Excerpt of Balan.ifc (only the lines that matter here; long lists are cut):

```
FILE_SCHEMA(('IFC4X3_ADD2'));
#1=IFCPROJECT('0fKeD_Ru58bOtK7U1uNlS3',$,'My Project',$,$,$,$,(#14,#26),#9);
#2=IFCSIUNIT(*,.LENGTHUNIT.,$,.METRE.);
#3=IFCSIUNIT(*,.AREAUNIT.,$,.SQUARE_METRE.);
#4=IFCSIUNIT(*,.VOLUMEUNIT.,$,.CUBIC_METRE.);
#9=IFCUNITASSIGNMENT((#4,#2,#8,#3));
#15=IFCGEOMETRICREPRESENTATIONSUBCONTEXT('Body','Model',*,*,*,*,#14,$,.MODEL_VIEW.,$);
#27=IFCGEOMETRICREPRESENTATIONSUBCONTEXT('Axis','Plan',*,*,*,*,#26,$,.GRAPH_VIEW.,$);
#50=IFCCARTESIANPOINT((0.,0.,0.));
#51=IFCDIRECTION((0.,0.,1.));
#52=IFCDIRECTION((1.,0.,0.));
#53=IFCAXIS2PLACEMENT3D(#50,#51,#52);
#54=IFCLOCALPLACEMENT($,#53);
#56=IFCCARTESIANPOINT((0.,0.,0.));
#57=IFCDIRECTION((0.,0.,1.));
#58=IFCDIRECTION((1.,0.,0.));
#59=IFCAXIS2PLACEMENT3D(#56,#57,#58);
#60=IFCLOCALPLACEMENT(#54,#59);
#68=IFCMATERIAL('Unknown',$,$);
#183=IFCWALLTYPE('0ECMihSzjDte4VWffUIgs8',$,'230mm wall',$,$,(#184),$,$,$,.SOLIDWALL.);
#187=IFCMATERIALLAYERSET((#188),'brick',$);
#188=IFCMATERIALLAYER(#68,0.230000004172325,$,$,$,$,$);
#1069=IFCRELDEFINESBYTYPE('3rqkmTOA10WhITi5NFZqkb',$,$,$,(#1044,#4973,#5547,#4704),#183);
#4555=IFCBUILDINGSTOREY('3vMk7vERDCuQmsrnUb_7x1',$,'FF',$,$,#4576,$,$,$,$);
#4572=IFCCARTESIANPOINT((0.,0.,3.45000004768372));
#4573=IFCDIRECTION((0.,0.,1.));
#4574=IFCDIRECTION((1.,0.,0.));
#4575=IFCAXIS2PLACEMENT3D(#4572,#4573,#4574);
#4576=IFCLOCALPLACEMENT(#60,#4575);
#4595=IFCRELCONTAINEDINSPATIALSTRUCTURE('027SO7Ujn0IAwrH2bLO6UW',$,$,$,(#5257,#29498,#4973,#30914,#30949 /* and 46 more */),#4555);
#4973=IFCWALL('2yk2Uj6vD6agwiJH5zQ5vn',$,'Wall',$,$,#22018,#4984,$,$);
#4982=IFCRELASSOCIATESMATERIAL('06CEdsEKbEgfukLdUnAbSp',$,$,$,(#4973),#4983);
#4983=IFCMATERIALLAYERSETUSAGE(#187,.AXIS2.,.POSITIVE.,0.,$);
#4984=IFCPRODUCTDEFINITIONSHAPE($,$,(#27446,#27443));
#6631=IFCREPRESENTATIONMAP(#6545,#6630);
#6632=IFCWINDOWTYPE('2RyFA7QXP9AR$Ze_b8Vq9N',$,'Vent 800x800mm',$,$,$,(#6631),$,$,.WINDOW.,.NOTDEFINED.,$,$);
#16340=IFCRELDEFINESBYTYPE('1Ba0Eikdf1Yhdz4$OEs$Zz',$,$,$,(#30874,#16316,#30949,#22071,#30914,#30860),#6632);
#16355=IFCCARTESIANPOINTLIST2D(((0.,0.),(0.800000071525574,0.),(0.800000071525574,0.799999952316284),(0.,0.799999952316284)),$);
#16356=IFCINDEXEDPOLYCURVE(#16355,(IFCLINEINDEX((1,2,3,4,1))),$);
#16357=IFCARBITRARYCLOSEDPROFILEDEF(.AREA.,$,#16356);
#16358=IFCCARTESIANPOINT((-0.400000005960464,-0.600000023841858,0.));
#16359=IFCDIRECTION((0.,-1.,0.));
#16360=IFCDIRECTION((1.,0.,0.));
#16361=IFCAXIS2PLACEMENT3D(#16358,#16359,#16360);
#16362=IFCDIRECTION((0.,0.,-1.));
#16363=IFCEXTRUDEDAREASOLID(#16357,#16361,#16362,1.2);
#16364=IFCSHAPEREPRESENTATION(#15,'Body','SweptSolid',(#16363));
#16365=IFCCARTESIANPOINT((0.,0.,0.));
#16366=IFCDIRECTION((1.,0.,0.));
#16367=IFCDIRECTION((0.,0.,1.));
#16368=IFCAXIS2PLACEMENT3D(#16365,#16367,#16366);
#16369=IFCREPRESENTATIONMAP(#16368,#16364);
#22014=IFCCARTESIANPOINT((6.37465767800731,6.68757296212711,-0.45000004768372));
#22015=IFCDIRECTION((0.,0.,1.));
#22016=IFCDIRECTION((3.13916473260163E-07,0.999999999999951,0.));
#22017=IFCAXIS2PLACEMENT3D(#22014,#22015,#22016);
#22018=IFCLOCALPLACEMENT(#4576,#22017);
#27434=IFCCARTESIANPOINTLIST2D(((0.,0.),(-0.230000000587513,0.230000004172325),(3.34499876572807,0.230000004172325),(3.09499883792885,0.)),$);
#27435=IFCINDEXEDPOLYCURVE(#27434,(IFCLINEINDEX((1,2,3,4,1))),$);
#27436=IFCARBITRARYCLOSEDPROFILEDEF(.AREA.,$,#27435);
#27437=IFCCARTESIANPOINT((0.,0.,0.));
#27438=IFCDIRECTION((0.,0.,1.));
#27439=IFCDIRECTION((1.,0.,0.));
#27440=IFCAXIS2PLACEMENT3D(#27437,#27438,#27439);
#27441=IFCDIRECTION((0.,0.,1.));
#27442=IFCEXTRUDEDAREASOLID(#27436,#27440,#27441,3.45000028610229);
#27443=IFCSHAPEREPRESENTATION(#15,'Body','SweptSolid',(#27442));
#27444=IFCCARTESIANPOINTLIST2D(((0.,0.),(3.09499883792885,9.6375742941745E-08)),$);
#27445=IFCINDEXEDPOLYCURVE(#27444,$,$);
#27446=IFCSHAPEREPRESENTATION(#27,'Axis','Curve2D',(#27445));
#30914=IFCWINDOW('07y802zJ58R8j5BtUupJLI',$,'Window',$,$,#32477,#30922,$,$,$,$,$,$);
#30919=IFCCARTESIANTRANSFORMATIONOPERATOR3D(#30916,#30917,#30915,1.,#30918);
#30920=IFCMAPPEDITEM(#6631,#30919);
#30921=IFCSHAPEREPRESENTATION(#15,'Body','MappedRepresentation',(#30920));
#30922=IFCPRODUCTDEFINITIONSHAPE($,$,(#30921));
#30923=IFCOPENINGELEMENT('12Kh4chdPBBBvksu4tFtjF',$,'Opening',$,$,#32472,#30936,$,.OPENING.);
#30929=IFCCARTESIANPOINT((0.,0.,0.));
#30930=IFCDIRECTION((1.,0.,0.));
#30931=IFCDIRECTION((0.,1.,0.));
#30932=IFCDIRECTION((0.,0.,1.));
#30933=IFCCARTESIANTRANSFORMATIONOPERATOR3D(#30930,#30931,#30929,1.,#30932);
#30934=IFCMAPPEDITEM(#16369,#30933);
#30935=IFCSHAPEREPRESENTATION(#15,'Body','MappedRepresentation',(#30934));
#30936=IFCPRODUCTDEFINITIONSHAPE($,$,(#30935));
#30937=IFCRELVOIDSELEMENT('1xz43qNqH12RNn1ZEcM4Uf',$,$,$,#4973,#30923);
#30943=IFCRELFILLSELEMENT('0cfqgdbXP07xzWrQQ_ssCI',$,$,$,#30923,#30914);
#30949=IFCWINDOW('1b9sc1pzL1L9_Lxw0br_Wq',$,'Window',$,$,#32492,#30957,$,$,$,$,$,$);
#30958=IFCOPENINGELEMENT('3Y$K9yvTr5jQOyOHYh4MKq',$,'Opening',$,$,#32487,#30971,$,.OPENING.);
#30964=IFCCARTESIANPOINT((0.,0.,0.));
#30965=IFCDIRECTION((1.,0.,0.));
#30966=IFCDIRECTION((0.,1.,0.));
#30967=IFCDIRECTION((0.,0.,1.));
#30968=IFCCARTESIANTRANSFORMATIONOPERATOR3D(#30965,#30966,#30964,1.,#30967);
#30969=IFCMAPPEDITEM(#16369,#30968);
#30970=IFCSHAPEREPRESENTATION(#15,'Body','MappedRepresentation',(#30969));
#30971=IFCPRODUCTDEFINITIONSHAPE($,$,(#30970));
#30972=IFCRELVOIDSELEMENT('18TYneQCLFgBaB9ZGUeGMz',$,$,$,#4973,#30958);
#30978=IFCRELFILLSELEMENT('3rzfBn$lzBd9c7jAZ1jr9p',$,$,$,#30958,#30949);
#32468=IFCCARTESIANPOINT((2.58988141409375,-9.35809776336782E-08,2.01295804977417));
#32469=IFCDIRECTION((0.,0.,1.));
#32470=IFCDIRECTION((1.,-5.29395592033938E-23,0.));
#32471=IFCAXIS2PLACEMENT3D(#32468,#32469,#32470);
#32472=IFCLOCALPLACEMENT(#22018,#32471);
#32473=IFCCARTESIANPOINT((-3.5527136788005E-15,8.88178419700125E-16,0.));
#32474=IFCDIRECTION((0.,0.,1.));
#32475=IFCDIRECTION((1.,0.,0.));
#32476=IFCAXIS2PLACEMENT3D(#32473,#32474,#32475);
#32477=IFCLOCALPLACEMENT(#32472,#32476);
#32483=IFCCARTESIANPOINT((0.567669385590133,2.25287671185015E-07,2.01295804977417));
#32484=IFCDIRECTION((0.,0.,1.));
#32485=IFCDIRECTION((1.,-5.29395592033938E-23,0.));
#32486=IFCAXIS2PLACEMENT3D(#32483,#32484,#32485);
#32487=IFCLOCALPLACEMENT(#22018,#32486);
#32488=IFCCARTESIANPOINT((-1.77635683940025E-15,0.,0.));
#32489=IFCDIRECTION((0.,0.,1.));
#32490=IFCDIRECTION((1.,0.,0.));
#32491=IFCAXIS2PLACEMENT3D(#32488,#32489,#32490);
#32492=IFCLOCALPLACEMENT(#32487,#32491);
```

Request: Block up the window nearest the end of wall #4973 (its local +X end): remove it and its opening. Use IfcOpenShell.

```python
import ifcopenshell
import ifcopenshell.api.feature
import ifcopenshell.api.root
import ifcopenshell.geom
import ifcopenshell.util.shape

model = ifcopenshell.open("Balan.ifc")
settings = ifcopenshell.geom.settings()


def volume(element):
    """Net volume in cubic metres, openings subtracted."""
    shape = ifcopenshell.geom.create_shape(settings, element)
    return ifcopenshell.util.shape.get_volume(shape.geometry)


window = model.by_id(30914)
opening = window.FillsVoids[0].RelatingOpeningElement
wall = opening.VoidsElements[0].RelatingBuildingElement
before = volume(wall)

ifcopenshell.api.root.remove_product(model, product=window)
ifcopenshell.api.feature.remove_feature(model, feature=opening)

after = volume(wall)

print(f"wall volume {before:.3f} -> {after:.3f} m3")

model.write("Balan-out.ifc")
```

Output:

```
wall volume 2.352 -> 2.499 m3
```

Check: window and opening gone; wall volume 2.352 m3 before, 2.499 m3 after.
